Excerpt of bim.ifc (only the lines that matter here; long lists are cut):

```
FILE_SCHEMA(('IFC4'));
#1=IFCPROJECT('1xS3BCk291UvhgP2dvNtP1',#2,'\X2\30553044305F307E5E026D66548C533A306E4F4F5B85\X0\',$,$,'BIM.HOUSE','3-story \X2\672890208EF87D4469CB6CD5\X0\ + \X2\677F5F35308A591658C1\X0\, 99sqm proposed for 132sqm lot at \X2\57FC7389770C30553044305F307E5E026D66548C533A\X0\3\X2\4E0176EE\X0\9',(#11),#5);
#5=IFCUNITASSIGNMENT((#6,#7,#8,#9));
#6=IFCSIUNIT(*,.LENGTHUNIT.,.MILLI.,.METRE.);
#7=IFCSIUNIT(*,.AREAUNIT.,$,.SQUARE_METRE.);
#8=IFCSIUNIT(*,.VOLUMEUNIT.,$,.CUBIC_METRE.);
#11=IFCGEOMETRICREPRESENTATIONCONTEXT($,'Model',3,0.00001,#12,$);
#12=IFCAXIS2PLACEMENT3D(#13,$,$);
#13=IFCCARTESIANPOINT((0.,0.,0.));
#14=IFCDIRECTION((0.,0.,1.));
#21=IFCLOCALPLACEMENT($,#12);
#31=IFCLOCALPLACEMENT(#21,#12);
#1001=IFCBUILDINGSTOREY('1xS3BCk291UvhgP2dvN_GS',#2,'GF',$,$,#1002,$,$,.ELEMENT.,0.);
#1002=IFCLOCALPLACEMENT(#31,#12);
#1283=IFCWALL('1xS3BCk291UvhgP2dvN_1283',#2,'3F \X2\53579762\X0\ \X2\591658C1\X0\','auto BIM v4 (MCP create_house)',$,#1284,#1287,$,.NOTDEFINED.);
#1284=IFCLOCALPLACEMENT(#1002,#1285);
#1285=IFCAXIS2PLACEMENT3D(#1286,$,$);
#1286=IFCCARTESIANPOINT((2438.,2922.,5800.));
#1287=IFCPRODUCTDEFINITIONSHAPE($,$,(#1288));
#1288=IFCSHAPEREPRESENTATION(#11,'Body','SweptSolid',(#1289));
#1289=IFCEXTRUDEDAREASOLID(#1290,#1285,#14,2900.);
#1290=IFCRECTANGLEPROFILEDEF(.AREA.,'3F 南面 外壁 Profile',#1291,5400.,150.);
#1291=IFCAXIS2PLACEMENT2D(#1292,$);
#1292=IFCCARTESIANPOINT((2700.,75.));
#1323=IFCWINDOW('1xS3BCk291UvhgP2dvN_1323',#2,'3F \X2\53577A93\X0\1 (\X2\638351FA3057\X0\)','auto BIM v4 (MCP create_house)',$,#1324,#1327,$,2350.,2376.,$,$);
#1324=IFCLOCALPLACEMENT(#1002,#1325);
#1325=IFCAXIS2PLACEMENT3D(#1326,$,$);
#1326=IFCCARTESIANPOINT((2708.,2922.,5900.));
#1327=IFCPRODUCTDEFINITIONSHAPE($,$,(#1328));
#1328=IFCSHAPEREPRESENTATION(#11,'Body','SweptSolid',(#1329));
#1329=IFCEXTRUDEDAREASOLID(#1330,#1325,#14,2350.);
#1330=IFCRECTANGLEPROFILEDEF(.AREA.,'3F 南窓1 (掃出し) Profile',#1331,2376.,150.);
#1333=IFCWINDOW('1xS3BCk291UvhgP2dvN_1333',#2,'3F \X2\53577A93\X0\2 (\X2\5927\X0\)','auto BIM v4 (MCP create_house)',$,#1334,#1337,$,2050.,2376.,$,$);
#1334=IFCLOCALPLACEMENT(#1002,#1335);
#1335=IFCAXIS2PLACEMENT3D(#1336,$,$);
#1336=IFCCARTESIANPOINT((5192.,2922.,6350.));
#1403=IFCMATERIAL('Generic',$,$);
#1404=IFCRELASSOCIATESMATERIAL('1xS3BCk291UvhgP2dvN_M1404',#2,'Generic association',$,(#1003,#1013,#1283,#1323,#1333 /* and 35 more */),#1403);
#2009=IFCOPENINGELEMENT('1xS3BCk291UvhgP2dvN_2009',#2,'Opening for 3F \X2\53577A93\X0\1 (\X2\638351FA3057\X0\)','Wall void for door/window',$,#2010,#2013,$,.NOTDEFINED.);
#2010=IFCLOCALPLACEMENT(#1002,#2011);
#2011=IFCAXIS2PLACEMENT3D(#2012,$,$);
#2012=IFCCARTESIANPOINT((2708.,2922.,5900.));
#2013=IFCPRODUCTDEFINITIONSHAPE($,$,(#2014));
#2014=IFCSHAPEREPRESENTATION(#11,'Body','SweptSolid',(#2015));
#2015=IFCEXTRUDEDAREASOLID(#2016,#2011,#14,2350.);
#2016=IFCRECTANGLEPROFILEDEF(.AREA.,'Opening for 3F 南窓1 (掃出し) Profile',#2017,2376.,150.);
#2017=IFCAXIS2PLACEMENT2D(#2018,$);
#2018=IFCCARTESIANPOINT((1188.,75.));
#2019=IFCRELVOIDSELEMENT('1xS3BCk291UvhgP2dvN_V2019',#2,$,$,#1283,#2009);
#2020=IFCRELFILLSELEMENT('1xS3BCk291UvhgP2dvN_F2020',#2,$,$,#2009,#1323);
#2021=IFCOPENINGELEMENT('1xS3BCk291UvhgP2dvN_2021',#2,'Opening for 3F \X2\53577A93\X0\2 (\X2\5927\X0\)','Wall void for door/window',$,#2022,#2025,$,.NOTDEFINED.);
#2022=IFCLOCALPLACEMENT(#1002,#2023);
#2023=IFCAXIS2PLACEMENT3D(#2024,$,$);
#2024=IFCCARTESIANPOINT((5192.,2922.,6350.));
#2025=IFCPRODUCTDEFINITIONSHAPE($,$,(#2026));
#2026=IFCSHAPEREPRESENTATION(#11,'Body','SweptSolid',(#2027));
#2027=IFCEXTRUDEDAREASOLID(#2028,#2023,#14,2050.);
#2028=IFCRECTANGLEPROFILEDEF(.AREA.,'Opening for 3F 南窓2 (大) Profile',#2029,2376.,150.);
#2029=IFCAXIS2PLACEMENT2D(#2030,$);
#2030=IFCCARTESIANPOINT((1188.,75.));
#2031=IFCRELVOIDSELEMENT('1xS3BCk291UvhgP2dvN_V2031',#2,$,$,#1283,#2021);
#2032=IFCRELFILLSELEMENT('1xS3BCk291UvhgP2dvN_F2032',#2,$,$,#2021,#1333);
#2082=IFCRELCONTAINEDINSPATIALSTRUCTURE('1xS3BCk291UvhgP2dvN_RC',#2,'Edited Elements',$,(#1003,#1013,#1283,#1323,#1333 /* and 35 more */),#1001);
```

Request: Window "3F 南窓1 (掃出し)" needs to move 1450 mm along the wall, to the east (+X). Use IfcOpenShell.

```python
import ifcopenshell
import ifcopenshell.api.geometry
import ifcopenshell.util.placement
import ifcopenshell.util.unit

model = ifcopenshell.open("bim.ifc")
unit_scale = ifcopenshell.util.unit.calculate_unit_scale(model)

window = model.by_guid("1xS3BCk291UvhgP2dvN_1323")
opening = window.FillsVoids[0].RelatingOpeningElement
wall = opening.VoidsElements[0].RelatingBuildingElement

wall_matrix = ifcopenshell.util.placement.get_local_placement(wall.ObjectPlacement)
shift = wall_matrix[:3, 0] * 1.45 / unit_scale
before = ifcopenshell.util.placement.get_local_placement(window.ObjectPlacement)[:3, 3].copy()

# The window is not placed relative to its opening, so move both.
for product in (opening, window):
    matrix = ifcopenshell.util.placement.get_local_placement(product.ObjectPlacement)
    matrix[:3, 3] += shift
    ifcopenshell.api.geometry.edit_object_placement(model, product=product, matrix=matrix, is_si=False)

after = ifcopenshell.util.placement.get_local_placement(window.ObjectPlacement)[:3, 3]
print("window moved by", (after - before).round(3) + 0.0)

model.write("bim_updated.ifc")
```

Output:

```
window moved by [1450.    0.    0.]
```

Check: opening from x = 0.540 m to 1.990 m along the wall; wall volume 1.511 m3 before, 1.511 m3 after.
